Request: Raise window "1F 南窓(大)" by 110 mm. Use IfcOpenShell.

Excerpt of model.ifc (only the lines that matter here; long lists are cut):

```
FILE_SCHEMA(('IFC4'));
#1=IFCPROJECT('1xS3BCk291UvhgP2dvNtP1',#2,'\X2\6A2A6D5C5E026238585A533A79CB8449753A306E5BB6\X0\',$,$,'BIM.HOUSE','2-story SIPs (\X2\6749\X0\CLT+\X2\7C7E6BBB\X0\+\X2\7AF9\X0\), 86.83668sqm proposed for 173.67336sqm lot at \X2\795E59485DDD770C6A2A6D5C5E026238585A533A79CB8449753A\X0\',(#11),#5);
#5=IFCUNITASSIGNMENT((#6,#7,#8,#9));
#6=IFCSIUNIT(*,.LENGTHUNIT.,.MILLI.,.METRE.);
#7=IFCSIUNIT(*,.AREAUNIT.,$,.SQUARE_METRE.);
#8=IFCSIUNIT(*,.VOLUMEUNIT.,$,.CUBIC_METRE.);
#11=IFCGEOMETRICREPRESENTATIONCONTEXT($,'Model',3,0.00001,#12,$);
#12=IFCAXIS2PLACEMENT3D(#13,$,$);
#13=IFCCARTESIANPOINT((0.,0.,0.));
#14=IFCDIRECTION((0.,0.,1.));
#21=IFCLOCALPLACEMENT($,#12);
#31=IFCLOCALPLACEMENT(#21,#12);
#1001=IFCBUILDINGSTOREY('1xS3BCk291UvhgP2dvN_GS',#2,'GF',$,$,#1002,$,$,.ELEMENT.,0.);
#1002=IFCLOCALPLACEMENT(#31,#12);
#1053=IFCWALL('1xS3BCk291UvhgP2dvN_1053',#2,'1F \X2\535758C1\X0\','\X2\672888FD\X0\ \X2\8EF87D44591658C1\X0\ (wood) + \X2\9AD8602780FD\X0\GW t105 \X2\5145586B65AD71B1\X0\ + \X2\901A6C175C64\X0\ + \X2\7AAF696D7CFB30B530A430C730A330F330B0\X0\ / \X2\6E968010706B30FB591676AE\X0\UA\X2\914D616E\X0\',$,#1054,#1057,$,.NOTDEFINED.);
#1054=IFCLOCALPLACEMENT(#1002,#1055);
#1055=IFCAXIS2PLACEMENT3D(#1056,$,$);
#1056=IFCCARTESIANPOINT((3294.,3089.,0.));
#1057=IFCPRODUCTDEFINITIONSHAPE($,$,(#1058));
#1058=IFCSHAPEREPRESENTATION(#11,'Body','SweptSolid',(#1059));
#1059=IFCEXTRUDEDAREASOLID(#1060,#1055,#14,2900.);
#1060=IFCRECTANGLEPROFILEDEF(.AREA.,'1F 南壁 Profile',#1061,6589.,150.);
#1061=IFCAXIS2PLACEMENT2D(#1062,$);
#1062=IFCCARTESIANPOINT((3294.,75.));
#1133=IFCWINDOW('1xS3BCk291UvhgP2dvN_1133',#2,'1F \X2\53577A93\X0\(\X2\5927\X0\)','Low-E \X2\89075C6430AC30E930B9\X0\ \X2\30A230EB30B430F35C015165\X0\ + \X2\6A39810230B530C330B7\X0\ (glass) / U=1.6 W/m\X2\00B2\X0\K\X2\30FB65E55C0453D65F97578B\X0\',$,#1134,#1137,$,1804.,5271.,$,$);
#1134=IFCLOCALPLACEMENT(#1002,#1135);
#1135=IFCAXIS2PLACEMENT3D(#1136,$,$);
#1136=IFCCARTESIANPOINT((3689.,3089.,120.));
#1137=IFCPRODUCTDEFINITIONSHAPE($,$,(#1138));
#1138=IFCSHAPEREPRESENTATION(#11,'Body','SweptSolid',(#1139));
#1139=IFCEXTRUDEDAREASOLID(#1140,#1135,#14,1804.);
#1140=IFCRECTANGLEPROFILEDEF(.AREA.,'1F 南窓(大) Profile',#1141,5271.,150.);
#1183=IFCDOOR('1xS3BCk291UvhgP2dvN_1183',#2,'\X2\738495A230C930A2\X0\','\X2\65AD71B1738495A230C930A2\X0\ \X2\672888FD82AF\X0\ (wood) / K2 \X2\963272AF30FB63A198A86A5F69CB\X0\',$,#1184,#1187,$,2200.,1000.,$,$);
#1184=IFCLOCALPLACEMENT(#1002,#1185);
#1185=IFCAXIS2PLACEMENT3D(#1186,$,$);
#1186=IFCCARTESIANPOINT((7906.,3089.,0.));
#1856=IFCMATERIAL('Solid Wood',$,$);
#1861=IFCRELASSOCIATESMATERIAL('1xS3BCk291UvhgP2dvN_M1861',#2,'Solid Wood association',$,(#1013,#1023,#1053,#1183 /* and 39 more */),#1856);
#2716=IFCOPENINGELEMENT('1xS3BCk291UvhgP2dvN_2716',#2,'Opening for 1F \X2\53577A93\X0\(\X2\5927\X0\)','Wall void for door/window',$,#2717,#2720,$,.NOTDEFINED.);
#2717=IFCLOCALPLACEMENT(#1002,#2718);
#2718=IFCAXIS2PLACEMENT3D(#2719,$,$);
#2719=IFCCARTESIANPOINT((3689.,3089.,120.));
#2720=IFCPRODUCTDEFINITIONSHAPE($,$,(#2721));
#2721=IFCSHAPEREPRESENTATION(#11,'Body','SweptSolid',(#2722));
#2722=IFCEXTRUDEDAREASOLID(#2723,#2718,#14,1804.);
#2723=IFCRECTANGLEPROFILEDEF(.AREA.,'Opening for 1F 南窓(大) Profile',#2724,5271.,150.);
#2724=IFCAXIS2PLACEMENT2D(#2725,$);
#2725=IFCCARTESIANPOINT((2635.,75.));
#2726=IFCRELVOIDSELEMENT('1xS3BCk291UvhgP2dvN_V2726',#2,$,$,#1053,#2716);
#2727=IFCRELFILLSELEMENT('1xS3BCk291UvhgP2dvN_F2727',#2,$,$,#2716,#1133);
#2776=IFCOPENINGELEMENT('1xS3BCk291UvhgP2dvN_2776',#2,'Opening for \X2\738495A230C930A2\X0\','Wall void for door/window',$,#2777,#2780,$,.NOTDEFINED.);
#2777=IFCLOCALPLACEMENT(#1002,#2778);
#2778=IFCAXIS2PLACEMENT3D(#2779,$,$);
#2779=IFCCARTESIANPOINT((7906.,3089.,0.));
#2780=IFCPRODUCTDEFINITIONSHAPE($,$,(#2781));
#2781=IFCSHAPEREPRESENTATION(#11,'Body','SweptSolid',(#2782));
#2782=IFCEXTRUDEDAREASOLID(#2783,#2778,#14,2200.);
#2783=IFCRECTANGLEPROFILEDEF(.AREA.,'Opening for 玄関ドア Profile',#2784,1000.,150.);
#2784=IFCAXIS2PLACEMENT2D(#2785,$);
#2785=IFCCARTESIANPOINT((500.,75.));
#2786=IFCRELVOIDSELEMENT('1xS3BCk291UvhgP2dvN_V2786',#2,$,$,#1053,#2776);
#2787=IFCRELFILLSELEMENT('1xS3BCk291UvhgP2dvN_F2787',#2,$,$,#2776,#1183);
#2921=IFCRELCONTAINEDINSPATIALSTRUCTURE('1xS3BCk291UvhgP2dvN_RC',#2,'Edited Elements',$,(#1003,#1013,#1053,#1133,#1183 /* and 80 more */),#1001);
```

```python
import numpy as np
import ifcopenshell
import ifcopenshell.api.geometry
import ifcopenshell.util.placement
import ifcopenshell.util.unit

model = ifcopenshell.open("model.ifc")
unit_scale = ifcopenshell.util.unit.calculate_unit_scale(model)

window = model.by_guid("1xS3BCk291UvhgP2dvN_1133")
opening = window.FillsVoids[0].RelatingOpeningElement
dz = 0.11 / unit_scale

shift = np.array([0.0, 0.0, dz])
# The window is not placed relative to its opening, so move both.
for product in (opening, window):
    matrix = ifcopenshell.util.placement.get_local_placement(product.ObjectPlacement)
    matrix[:3, 3] += shift
    ifcopenshell.api.geometry.edit_object_placement(model, product=product, matrix=matrix, is_si=False)

print(f"moved by {dz * unit_scale:+.3f} m")

model.write("model-out.ifc")
```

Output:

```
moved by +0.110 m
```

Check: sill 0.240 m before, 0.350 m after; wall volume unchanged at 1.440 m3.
